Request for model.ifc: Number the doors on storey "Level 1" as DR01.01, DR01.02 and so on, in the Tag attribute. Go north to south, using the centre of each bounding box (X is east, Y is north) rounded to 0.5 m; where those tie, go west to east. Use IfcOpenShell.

First a look at what the model holds.

```python
import ifcopenshell
import ifcopenshell.util.element
import ifcopenshell.util.placement

model = ifcopenshell.open("model.ifc")
print(model.schema)
storey = next(s for s in model.by_type("IfcBuildingStorey") if s.Name == "Level 1")
doors = [e for e in ifcopenshell.util.element.get_decomposition(storey) if e.is_a("IfcDoor")]
for e in sorted(doors, key=lambda e: e.id()):
    origin = ifcopenshell.util.placement.get_local_placement(e.ObjectPlacement)[:3, 3]
    print(e.id(), e.Tag, e.Name, origin.round(2) + 0.0, sep=" | ")
```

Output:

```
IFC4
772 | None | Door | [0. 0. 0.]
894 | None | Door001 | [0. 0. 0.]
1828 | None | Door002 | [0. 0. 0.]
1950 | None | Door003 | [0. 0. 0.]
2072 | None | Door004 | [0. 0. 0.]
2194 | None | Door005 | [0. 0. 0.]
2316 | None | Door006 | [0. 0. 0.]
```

```python
import ifcopenshell
import ifcopenshell.geom
import ifcopenshell.util.element
import ifcopenshell.util.shape

model = ifcopenshell.open("model.ifc")
settings = ifcopenshell.geom.settings()
settings.set("use-world-coords", True)


def centre(element):
    shape = ifcopenshell.geom.create_shape(settings, element)
    return ifcopenshell.util.shape.get_bbox_centroid(shape.geometry)


storey = next(s for s in model.by_type("IfcBuildingStorey") if s.Name == "Level 1")
doors = [e for e in ifcopenshell.util.element.get_decomposition(storey) if e.is_a("IfcDoor")]

# Insertion points can sit at a corner or the storey origin, so sort by the geometry (in metres).
centres = {e: centre(e) for e in doors}
doors.sort(key=lambda e: (-round(centres[e][1] / 0.5), centres[e][0]))

for i, e in enumerate(doors, start=1):
    number = f"DR01.{i:02d}"
    e.Tag = number
    print(e.id(), number)

model.write("model_rev.ifc")
```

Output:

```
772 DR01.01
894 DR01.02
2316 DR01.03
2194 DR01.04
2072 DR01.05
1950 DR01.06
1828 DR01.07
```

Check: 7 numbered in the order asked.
